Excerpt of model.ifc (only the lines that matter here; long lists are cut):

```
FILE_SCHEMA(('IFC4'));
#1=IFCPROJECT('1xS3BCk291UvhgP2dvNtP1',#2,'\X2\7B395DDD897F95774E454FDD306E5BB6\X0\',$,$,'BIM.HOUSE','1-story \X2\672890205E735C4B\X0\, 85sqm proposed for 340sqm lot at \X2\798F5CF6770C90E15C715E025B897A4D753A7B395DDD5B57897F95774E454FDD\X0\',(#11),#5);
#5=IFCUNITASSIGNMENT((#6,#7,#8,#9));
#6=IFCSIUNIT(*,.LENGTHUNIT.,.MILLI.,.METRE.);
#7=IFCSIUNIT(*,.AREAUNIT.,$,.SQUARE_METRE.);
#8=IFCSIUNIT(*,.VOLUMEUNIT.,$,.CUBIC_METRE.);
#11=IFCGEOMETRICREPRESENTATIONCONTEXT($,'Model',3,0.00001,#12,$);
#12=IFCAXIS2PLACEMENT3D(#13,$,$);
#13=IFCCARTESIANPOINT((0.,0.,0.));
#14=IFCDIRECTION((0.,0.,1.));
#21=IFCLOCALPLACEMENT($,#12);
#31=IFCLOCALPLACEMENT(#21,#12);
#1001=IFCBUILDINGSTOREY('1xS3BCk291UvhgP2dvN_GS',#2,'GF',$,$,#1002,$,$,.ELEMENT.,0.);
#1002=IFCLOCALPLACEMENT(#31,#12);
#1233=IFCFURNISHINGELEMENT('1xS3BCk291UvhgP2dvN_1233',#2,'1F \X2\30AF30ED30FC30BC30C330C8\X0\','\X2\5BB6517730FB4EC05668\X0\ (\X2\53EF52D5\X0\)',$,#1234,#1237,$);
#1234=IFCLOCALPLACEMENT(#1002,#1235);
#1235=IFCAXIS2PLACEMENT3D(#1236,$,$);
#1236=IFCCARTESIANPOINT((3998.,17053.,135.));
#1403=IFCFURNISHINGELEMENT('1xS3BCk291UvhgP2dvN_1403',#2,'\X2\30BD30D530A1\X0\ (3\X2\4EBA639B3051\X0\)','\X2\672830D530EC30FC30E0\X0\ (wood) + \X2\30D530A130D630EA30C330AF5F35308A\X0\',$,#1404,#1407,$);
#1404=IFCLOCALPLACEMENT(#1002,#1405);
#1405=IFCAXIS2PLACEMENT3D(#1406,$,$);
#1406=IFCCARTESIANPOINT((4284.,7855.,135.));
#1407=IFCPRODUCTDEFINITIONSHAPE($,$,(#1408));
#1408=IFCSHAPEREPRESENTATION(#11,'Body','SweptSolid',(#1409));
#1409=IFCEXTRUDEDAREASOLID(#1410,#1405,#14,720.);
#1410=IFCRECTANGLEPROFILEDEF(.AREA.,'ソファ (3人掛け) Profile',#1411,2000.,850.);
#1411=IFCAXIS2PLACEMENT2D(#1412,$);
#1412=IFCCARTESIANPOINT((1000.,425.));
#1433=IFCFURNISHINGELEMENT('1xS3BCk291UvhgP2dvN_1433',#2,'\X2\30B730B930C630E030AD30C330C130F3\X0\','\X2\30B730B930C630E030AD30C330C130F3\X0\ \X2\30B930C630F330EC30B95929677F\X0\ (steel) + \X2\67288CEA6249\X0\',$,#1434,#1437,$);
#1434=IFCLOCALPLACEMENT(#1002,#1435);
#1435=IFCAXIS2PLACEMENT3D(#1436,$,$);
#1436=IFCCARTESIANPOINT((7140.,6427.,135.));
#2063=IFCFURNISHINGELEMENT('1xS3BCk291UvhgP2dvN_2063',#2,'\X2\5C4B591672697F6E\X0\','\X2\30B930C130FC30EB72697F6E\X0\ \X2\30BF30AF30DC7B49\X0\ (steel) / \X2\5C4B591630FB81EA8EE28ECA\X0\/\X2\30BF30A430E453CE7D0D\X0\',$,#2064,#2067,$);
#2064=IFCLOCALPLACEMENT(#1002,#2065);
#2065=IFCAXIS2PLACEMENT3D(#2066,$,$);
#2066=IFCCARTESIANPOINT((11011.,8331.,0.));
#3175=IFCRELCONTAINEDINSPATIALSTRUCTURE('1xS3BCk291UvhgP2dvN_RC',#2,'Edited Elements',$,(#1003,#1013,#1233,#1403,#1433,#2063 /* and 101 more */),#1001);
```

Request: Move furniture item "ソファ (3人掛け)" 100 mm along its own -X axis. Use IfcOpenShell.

```python
import ifcopenshell
import ifcopenshell.api.geometry
import ifcopenshell.util.placement

model = ifcopenshell.open("model.ifc")

item = model.by_guid("1xS3BCk291UvhgP2dvN_1403")
matrix = ifcopenshell.util.placement.get_local_placement(item.ObjectPlacement)
matrix[:3, 3] -= matrix[:3, 0] * 100.0
ifcopenshell.api.geometry.edit_object_placement(model, product=item, matrix=matrix, is_si=False)

print(ifcopenshell.util.placement.get_local_placement(item.ObjectPlacement).round(3) + 0.0)

model.write("model_edited.ifc")
```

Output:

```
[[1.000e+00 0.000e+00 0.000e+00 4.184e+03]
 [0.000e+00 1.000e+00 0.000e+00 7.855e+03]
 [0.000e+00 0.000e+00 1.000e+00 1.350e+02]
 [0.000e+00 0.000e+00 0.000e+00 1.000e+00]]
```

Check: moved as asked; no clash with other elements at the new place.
